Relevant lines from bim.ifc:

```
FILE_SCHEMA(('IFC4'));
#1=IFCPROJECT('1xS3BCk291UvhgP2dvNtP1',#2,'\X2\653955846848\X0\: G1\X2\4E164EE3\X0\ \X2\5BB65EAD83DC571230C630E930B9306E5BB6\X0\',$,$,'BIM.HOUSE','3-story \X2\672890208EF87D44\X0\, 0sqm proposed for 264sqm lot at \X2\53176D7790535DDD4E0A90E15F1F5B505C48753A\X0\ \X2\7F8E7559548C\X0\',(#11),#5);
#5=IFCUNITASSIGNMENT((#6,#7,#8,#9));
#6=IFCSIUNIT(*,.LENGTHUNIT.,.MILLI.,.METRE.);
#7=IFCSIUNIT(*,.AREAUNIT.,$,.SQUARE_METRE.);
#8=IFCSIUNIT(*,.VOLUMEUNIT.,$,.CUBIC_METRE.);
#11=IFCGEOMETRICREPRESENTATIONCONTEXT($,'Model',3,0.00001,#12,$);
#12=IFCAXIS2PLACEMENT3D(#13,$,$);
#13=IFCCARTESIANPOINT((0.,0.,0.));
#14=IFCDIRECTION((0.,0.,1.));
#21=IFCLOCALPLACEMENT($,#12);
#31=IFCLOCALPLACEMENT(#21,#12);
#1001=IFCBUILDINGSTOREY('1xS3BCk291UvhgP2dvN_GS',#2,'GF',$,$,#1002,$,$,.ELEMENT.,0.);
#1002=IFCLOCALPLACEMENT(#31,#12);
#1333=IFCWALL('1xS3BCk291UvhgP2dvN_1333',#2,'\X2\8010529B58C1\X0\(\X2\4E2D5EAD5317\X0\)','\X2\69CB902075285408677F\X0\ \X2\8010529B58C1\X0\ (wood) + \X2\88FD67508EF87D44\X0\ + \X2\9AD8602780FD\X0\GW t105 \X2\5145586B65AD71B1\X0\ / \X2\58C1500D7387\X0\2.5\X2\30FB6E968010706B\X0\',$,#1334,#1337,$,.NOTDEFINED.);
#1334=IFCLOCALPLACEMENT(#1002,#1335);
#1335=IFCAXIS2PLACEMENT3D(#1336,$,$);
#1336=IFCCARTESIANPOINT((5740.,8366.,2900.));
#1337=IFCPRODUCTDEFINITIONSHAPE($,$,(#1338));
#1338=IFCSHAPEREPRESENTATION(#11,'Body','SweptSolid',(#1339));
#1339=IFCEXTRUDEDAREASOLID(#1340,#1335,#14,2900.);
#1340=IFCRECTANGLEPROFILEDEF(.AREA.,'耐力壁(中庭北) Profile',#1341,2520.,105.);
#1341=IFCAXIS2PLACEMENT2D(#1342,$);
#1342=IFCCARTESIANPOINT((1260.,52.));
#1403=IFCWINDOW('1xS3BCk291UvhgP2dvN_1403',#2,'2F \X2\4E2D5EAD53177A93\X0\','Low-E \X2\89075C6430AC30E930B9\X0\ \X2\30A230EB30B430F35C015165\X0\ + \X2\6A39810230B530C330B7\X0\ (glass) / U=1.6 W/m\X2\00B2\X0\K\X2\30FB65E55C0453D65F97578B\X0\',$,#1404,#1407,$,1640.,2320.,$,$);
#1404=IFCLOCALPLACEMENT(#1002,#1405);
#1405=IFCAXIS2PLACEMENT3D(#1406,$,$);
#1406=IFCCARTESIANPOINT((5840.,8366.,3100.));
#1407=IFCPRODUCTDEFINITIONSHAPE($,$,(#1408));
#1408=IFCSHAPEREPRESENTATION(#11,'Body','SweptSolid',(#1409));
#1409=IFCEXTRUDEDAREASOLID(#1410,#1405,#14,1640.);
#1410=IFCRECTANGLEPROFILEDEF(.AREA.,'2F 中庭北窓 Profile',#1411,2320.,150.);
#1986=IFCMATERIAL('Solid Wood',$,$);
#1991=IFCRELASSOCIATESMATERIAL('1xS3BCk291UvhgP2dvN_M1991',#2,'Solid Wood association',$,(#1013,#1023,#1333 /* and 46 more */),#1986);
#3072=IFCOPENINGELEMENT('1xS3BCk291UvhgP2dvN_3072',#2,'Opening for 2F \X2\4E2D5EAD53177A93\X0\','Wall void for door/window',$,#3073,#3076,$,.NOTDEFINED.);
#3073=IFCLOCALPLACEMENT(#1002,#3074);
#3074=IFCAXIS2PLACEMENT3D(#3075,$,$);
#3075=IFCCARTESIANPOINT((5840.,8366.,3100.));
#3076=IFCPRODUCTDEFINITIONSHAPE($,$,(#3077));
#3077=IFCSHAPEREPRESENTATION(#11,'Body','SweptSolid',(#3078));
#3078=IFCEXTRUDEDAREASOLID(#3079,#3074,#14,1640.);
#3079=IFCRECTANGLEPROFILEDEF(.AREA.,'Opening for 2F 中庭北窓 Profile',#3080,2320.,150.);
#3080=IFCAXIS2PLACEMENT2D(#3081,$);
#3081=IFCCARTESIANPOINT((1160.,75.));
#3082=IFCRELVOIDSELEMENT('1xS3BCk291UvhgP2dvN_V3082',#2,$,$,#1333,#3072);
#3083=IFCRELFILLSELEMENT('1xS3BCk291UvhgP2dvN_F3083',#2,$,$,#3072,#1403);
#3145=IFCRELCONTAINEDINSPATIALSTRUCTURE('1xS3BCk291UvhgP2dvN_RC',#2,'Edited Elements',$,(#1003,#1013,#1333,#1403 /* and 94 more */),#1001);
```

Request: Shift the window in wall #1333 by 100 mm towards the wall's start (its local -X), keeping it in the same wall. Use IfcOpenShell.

```python
import ifcopenshell
import ifcopenshell.api.geometry
import ifcopenshell.util.placement

model = ifcopenshell.open("bim.ifc")

window = model.by_guid("1xS3BCk291UvhgP2dvN_1403")
opening = window.FillsVoids[0].RelatingOpeningElement
wall = opening.VoidsElements[0].RelatingBuildingElement

wall_matrix = ifcopenshell.util.placement.get_local_placement(wall.ObjectPlacement)
shift = wall_matrix[:3, 0] * -100.0
before = ifcopenshell.util.placement.get_local_placement(window.ObjectPlacement)[:3, 3].copy()

# The window is not placed relative to its opening, so move both.
for product in (opening, window):
    matrix = ifcopenshell.util.placement.get_local_placement(product.ObjectPlacement)
    matrix[:3, 3] += shift
    ifcopenshell.api.geometry.edit_object_placement(model, product=product, matrix=matrix, is_si=False)

after = ifcopenshell.util.placement.get_local_placement(window.ObjectPlacement)[:3, 3]
print("window moved by", (after - before).round(3) + 0.0)

model.write("bim_v2.ifc")
```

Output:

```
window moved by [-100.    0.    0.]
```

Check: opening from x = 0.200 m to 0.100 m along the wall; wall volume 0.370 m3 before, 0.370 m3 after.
